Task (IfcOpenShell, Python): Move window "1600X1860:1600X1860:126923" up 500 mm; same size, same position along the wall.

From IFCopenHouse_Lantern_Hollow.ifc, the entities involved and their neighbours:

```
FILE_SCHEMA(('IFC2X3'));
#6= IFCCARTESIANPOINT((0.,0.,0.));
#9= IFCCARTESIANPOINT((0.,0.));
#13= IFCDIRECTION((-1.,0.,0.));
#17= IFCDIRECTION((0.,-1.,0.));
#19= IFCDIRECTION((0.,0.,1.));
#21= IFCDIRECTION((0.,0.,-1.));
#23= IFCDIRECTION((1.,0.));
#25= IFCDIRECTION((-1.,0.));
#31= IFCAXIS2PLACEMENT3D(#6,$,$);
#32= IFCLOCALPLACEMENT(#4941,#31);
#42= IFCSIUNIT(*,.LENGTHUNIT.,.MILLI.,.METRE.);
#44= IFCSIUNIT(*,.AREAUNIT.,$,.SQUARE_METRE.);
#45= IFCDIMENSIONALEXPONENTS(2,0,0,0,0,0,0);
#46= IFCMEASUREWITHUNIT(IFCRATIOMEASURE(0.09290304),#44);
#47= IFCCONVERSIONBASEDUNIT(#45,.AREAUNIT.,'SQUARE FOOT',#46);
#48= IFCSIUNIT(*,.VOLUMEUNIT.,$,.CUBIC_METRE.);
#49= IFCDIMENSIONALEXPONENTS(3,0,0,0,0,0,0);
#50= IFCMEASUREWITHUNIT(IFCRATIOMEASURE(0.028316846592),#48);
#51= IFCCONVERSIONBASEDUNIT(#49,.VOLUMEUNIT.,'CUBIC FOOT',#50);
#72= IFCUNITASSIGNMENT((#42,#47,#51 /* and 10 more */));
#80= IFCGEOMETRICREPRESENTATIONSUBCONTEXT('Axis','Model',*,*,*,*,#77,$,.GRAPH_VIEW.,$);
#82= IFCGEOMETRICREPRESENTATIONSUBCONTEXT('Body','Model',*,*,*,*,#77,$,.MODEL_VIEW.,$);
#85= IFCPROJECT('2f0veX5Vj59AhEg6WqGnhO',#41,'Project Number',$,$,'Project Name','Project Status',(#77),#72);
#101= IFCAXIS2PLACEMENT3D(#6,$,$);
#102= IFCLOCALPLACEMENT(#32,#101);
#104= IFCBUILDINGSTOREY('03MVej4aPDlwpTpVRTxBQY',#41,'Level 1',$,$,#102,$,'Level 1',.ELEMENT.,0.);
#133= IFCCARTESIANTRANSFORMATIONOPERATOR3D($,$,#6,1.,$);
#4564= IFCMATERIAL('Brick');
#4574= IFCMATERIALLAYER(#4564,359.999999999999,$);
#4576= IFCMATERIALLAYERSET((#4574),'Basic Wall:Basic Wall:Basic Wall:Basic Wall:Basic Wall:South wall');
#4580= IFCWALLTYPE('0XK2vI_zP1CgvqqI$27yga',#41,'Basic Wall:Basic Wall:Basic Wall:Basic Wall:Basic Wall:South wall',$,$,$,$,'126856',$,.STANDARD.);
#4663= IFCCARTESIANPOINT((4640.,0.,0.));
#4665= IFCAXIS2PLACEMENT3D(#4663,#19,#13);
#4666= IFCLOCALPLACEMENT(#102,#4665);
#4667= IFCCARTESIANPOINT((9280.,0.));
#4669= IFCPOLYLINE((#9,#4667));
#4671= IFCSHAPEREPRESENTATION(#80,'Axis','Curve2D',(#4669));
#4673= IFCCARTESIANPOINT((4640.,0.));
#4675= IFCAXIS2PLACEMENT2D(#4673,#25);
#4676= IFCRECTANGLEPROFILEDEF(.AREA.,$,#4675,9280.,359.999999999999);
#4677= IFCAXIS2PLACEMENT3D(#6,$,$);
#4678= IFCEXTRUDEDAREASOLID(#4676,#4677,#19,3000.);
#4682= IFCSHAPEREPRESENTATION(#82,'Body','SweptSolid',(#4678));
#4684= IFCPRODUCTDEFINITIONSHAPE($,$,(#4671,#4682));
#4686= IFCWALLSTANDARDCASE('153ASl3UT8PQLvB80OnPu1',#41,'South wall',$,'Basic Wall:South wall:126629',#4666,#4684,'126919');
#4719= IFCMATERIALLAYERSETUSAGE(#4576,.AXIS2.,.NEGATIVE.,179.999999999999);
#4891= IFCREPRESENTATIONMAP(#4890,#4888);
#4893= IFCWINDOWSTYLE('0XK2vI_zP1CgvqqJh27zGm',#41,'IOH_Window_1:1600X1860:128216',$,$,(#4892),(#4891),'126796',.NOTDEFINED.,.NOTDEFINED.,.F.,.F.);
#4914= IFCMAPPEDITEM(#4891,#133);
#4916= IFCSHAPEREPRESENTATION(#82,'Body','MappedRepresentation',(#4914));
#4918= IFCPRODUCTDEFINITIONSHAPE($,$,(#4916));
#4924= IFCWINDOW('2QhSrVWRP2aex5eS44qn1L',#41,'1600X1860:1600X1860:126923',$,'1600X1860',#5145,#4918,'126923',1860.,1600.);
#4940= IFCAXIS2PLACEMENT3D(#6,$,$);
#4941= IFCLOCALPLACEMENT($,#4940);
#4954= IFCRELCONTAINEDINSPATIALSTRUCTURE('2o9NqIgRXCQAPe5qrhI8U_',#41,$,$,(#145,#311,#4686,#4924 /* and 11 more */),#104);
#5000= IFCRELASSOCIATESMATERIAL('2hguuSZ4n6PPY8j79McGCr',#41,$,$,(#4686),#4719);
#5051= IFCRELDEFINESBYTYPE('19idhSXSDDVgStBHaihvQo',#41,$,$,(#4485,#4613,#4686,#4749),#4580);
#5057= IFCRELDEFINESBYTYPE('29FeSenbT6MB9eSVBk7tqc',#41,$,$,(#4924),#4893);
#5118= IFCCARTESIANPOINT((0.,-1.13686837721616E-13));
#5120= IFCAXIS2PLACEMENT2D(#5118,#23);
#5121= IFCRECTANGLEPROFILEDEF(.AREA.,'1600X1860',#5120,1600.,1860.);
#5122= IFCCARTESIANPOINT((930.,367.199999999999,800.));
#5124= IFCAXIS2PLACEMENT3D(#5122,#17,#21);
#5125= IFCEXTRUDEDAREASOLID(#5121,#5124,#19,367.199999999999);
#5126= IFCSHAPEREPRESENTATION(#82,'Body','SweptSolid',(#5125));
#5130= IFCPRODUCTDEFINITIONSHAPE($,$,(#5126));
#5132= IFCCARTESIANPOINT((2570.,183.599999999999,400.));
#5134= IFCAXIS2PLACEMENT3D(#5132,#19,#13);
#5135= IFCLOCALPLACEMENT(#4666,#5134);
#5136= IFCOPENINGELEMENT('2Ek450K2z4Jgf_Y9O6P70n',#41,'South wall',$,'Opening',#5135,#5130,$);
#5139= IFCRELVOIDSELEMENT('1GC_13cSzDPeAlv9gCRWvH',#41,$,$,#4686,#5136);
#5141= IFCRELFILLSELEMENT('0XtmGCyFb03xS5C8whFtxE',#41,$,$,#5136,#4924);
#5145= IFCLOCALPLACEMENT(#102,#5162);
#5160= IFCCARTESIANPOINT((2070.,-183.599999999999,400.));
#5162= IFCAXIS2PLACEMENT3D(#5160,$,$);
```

```python
import numpy as np
import ifcopenshell
import ifcopenshell.api.geometry
import ifcopenshell.util.placement
import ifcopenshell.util.unit

model = ifcopenshell.open("IFCopenHouse_Lantern_Hollow.ifc")
unit_scale = ifcopenshell.util.unit.calculate_unit_scale(model)

window = model.by_guid("2QhSrVWRP2aex5eS44qn1L")
opening = window.FillsVoids[0].RelatingOpeningElement
dz = 0.5 / unit_scale

shift = np.array([0.0, 0.0, dz])
# The window is not placed relative to its opening, so move both.
for product in (opening, window):
    matrix = ifcopenshell.util.placement.get_local_placement(product.ObjectPlacement)
    matrix[:3, 3] += shift
    ifcopenshell.api.geometry.edit_object_placement(model, product=product, matrix=matrix, is_si=False)

print(f"moved by {dz * unit_scale:+.3f} m")

model.write("IFCopenHouse_Lantern_Hollow_edited.ifc")
```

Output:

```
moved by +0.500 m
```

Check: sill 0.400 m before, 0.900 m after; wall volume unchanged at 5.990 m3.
